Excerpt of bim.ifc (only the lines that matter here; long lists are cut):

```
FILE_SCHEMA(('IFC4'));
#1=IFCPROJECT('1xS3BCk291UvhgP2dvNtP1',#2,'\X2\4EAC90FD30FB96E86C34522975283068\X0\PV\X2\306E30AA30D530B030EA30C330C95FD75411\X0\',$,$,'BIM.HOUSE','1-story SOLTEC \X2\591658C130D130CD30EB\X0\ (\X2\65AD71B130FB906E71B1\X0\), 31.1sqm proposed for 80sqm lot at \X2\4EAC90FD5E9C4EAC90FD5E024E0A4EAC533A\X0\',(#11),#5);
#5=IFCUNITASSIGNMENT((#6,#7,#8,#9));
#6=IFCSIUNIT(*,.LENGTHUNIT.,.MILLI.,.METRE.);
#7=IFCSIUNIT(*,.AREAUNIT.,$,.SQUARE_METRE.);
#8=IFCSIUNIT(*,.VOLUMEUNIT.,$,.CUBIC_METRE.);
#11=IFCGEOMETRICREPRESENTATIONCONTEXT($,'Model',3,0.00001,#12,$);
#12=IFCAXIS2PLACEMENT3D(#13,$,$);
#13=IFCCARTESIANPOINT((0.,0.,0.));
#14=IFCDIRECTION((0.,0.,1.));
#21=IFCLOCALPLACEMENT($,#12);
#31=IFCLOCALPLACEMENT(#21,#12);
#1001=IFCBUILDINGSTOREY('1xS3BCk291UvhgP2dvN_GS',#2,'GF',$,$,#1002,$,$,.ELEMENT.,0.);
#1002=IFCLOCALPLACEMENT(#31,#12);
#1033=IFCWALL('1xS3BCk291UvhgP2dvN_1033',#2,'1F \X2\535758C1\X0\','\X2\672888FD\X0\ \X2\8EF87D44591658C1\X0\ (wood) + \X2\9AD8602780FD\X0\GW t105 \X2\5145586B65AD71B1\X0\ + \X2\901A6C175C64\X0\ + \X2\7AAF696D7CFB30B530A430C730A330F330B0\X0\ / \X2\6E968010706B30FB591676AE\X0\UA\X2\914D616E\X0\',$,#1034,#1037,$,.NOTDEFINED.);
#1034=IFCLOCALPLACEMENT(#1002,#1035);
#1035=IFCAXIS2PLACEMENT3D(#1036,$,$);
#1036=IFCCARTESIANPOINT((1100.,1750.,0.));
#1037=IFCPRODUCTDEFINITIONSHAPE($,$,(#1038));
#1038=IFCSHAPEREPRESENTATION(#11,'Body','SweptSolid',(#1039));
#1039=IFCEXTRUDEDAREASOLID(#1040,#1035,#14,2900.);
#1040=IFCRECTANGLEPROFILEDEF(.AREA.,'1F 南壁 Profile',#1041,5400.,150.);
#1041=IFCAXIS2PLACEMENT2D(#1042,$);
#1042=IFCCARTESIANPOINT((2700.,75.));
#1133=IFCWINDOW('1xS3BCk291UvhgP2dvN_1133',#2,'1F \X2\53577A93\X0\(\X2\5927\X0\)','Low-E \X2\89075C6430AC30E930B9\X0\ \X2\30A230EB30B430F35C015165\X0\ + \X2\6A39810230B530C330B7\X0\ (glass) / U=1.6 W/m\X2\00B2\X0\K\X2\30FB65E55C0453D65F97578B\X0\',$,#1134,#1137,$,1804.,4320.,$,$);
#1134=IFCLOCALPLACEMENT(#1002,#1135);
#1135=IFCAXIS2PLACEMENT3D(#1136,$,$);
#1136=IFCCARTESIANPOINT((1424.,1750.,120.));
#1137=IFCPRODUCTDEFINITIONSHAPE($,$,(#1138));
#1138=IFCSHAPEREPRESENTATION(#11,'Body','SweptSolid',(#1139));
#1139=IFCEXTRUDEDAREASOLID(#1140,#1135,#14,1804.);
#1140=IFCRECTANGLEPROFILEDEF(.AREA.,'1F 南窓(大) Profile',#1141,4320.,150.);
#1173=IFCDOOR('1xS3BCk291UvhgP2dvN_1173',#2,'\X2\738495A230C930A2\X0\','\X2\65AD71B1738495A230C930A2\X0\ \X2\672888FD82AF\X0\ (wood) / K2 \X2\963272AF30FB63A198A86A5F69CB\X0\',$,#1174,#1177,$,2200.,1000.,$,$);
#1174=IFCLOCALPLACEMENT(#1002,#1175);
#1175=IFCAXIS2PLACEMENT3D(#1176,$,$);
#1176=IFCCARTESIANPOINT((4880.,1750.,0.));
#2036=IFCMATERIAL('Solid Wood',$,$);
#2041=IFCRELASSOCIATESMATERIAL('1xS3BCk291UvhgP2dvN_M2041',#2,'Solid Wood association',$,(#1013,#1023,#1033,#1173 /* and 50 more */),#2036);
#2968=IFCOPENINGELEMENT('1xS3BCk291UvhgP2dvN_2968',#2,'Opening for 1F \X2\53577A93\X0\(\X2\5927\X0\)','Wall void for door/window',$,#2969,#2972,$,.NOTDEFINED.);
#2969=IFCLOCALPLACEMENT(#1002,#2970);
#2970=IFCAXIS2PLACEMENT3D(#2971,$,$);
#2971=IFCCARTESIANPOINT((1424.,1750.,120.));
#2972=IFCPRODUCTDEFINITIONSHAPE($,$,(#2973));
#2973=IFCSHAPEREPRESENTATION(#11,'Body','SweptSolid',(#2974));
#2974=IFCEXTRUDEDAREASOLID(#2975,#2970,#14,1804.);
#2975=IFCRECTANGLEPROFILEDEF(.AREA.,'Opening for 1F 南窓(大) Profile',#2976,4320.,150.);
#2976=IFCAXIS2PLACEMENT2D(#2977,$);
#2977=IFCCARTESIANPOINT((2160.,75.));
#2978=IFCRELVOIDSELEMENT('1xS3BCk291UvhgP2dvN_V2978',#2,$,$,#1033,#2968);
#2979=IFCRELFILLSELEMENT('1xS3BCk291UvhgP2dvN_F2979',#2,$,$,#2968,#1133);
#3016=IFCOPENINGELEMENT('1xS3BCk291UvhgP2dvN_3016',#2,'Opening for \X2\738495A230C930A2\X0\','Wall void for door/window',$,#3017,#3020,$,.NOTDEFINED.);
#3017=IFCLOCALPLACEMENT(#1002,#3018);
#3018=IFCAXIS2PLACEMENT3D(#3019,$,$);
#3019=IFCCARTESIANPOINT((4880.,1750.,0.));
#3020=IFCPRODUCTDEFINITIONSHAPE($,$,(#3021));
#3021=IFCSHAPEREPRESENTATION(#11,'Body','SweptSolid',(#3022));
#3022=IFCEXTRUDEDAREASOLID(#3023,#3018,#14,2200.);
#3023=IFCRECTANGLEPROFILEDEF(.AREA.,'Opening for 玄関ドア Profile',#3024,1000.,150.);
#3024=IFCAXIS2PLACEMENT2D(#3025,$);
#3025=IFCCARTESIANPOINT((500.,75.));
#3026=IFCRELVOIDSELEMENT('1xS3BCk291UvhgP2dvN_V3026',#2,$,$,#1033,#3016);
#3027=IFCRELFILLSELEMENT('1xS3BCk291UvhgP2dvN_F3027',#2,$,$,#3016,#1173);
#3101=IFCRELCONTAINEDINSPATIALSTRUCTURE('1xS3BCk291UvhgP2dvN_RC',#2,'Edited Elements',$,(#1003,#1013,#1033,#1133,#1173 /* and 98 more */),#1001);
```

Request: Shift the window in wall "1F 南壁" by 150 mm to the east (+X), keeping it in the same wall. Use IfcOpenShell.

```python
import ifcopenshell
import ifcopenshell.api.geometry
import ifcopenshell.util.placement
import ifcopenshell.util.unit

model = ifcopenshell.open("bim.ifc")
unit_scale = ifcopenshell.util.unit.calculate_unit_scale(model)

window = model.by_guid("1xS3BCk291UvhgP2dvN_1133")
opening = window.FillsVoids[0].RelatingOpeningElement
wall = opening.VoidsElements[0].RelatingBuildingElement

wall_matrix = ifcopenshell.util.placement.get_local_placement(wall.ObjectPlacement)
shift = wall_matrix[:3, 0] * 0.15 / unit_scale
before = ifcopenshell.util.placement.get_local_placement(window.ObjectPlacement)[:3, 3].copy()

# The window is not placed relative to its opening, so move both.
for product in (opening, window):
    matrix = ifcopenshell.util.placement.get_local_placement(product.ObjectPlacement)
    matrix[:3, 3] += shift
    ifcopenshell.api.geometry.edit_object_placement(model, product=product, matrix=matrix, is_si=False)

after = ifcopenshell.util.placement.get_local_placement(window.ObjectPlacement)[:3, 3]
print("window moved by", (after - before).round(3) + 0.0)

model.write("bim_v2.ifc")
```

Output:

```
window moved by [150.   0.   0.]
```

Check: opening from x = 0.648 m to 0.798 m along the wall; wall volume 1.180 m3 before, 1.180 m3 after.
